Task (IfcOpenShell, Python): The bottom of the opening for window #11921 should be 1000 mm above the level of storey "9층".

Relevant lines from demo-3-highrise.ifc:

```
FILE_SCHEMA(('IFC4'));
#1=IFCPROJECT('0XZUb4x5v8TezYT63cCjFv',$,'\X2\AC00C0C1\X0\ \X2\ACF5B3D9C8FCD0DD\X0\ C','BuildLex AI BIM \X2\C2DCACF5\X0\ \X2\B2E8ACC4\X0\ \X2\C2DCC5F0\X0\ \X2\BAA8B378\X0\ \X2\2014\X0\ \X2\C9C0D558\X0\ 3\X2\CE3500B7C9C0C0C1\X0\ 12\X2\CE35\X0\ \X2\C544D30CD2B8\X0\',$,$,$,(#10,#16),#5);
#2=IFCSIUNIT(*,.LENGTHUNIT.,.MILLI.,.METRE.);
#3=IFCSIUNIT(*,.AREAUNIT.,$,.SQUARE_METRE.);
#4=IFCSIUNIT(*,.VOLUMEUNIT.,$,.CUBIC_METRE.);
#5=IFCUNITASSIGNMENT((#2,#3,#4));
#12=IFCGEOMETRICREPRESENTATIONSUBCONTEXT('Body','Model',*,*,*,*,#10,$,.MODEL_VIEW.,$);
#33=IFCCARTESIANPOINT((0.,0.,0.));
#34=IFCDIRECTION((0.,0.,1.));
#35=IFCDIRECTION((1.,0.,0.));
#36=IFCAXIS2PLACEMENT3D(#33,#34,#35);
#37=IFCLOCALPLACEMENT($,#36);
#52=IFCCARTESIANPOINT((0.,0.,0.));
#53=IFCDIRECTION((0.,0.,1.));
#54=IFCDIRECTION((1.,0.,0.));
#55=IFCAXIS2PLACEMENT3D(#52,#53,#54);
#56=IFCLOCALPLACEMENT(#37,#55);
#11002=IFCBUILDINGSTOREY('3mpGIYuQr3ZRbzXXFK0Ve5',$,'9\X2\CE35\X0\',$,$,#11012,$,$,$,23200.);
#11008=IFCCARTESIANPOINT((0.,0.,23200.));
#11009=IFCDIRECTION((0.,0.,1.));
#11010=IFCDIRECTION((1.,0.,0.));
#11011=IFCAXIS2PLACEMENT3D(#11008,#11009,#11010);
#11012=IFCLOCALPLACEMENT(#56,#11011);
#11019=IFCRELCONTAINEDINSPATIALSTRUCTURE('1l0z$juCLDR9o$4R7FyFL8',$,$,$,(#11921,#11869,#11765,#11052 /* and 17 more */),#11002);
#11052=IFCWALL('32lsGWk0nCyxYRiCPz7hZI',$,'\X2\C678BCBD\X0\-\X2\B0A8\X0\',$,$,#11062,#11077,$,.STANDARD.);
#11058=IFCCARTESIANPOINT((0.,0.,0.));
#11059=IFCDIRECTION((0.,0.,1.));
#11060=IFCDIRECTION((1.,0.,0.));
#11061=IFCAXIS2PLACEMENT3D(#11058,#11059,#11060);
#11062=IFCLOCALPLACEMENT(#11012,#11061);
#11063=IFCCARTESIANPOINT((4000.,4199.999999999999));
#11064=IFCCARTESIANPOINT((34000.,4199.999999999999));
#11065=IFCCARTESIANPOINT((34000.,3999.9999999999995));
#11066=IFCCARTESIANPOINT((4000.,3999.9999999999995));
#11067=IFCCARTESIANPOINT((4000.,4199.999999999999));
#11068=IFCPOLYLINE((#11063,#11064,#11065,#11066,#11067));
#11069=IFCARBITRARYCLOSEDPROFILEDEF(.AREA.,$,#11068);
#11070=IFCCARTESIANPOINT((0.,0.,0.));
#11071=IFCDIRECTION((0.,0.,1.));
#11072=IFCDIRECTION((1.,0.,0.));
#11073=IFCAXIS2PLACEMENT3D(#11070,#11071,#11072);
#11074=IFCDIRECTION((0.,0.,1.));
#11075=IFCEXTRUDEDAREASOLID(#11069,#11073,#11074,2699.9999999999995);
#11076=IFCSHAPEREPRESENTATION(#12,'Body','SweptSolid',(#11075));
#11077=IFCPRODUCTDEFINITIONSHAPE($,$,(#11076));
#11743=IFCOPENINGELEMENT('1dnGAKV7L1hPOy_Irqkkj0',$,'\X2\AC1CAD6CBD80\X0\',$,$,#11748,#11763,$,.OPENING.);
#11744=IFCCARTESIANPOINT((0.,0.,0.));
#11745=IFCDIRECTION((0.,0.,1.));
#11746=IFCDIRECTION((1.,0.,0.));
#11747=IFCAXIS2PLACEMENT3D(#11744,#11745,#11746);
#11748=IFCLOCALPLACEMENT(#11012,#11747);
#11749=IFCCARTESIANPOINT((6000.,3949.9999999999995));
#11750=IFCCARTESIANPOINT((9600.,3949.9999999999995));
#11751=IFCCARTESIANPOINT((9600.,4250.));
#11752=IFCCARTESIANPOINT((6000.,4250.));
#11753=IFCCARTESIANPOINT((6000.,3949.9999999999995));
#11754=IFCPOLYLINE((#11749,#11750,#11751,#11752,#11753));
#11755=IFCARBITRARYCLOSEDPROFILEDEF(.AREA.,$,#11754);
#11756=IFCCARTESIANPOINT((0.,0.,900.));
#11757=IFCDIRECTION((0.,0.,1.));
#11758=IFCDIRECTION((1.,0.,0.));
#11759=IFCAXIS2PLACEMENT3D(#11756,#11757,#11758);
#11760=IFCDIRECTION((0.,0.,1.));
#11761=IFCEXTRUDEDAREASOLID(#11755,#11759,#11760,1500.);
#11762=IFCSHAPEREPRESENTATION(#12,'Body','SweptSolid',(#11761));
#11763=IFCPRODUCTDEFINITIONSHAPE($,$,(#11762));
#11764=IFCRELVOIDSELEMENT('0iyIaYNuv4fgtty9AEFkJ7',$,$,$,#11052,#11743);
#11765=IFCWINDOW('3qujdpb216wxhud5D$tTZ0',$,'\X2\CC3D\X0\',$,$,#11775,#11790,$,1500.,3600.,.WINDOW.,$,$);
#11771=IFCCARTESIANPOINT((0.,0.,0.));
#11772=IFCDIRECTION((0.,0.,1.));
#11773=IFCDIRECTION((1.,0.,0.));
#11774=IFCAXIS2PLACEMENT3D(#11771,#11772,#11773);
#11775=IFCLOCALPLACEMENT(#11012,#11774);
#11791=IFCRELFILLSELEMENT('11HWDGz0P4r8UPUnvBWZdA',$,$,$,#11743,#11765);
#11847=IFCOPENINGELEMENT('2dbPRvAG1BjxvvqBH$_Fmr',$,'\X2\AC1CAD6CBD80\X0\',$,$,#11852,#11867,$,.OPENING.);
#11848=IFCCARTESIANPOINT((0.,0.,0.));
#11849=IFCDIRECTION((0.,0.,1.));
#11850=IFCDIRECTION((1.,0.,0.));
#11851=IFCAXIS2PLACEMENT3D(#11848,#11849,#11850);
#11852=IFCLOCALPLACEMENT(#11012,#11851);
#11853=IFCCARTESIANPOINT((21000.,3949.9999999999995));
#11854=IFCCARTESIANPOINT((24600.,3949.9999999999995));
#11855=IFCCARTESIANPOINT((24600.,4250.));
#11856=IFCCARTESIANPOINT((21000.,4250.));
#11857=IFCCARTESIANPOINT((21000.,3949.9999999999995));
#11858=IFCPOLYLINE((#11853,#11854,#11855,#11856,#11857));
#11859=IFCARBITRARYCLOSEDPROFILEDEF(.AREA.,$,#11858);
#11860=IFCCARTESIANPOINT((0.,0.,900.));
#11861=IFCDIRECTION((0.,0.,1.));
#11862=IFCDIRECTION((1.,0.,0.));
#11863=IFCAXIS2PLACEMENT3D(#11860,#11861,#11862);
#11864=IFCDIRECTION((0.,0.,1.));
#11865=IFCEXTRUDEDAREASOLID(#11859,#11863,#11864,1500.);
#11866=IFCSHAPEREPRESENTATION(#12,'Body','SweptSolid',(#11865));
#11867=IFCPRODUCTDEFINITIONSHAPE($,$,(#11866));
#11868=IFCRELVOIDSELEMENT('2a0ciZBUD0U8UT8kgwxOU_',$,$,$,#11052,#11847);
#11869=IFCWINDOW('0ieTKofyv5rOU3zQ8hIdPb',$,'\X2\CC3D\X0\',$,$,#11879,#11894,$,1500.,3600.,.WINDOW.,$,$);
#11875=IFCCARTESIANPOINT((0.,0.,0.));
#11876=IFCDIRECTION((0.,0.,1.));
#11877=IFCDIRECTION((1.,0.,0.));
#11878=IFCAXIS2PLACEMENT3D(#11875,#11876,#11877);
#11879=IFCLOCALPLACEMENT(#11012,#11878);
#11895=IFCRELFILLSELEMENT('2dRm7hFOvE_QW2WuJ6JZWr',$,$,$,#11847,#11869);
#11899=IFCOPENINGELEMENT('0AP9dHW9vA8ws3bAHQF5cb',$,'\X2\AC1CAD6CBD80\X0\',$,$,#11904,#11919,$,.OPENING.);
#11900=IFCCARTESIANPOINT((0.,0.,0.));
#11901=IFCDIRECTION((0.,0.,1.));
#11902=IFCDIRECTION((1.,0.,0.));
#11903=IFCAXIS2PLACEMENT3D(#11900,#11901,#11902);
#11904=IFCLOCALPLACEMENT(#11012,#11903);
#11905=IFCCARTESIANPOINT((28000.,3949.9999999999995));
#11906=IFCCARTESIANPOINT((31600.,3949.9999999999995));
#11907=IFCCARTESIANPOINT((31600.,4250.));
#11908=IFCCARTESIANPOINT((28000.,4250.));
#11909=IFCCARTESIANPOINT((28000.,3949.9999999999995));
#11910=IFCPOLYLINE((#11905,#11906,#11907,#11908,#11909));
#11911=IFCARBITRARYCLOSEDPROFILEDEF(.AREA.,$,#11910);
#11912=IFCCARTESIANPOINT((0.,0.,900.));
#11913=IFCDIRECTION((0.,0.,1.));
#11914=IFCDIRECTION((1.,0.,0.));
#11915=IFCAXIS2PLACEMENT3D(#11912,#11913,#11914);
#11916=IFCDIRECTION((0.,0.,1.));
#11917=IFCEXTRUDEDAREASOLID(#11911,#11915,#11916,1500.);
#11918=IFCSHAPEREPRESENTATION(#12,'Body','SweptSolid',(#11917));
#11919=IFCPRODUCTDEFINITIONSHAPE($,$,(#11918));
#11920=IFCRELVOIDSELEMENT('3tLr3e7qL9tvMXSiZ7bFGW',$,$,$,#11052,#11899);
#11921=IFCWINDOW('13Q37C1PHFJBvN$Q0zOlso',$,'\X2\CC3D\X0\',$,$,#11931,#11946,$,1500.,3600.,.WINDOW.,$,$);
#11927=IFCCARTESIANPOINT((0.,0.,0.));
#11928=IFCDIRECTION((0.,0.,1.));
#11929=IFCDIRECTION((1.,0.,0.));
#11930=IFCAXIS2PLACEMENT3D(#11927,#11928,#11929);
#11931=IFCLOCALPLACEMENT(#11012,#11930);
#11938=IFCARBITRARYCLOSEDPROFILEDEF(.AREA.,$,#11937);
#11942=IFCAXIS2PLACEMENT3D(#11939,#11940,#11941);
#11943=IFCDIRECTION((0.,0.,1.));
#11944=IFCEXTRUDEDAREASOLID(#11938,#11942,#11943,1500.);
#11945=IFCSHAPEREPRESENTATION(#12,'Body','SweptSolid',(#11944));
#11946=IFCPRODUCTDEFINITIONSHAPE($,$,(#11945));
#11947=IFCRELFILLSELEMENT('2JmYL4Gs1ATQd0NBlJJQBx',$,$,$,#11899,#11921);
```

```python
import numpy as np
import ifcopenshell
import ifcopenshell.api.geometry
import ifcopenshell.geom
import ifcopenshell.util.element
import ifcopenshell.util.placement
import ifcopenshell.util.shape
import ifcopenshell.util.unit

model = ifcopenshell.open("demo-3-highrise.ifc")
unit_scale = ifcopenshell.util.unit.calculate_unit_scale(model)

window = model.by_guid("13Q37C1PHFJBvN$Q0zOlso")
opening = window.FillsVoids[0].RelatingOpeningElement
storey = ifcopenshell.util.element.get_container(window, ifc_class="IfcBuildingStorey")
level = ifcopenshell.util.placement.get_local_placement(storey.ObjectPlacement)[2, 3]

# The opening's origin need not be at the sill, so measure its lowest point.
shape = ifcopenshell.geom.create_shape(ifcopenshell.geom.settings(), opening)
bottom = ifcopenshell.util.shape.get_shape_bottom_elevation(shape, shape.geometry) / unit_scale
dz = level + 1 / unit_scale - bottom

shift = np.array([0.0, 0.0, dz])
# The window is not placed relative to its opening, so move both.
for product in (opening, window):
    matrix = ifcopenshell.util.placement.get_local_placement(product.ObjectPlacement)
    matrix[:3, 3] += shift
    ifcopenshell.api.geometry.edit_object_placement(model, product=product, matrix=matrix, is_si=False)

print(f"moved by {dz * unit_scale:+.3f} m")

model.write("demo-3-highrise_rev.ifc")
```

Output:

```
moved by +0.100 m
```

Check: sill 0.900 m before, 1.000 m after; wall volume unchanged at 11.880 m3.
